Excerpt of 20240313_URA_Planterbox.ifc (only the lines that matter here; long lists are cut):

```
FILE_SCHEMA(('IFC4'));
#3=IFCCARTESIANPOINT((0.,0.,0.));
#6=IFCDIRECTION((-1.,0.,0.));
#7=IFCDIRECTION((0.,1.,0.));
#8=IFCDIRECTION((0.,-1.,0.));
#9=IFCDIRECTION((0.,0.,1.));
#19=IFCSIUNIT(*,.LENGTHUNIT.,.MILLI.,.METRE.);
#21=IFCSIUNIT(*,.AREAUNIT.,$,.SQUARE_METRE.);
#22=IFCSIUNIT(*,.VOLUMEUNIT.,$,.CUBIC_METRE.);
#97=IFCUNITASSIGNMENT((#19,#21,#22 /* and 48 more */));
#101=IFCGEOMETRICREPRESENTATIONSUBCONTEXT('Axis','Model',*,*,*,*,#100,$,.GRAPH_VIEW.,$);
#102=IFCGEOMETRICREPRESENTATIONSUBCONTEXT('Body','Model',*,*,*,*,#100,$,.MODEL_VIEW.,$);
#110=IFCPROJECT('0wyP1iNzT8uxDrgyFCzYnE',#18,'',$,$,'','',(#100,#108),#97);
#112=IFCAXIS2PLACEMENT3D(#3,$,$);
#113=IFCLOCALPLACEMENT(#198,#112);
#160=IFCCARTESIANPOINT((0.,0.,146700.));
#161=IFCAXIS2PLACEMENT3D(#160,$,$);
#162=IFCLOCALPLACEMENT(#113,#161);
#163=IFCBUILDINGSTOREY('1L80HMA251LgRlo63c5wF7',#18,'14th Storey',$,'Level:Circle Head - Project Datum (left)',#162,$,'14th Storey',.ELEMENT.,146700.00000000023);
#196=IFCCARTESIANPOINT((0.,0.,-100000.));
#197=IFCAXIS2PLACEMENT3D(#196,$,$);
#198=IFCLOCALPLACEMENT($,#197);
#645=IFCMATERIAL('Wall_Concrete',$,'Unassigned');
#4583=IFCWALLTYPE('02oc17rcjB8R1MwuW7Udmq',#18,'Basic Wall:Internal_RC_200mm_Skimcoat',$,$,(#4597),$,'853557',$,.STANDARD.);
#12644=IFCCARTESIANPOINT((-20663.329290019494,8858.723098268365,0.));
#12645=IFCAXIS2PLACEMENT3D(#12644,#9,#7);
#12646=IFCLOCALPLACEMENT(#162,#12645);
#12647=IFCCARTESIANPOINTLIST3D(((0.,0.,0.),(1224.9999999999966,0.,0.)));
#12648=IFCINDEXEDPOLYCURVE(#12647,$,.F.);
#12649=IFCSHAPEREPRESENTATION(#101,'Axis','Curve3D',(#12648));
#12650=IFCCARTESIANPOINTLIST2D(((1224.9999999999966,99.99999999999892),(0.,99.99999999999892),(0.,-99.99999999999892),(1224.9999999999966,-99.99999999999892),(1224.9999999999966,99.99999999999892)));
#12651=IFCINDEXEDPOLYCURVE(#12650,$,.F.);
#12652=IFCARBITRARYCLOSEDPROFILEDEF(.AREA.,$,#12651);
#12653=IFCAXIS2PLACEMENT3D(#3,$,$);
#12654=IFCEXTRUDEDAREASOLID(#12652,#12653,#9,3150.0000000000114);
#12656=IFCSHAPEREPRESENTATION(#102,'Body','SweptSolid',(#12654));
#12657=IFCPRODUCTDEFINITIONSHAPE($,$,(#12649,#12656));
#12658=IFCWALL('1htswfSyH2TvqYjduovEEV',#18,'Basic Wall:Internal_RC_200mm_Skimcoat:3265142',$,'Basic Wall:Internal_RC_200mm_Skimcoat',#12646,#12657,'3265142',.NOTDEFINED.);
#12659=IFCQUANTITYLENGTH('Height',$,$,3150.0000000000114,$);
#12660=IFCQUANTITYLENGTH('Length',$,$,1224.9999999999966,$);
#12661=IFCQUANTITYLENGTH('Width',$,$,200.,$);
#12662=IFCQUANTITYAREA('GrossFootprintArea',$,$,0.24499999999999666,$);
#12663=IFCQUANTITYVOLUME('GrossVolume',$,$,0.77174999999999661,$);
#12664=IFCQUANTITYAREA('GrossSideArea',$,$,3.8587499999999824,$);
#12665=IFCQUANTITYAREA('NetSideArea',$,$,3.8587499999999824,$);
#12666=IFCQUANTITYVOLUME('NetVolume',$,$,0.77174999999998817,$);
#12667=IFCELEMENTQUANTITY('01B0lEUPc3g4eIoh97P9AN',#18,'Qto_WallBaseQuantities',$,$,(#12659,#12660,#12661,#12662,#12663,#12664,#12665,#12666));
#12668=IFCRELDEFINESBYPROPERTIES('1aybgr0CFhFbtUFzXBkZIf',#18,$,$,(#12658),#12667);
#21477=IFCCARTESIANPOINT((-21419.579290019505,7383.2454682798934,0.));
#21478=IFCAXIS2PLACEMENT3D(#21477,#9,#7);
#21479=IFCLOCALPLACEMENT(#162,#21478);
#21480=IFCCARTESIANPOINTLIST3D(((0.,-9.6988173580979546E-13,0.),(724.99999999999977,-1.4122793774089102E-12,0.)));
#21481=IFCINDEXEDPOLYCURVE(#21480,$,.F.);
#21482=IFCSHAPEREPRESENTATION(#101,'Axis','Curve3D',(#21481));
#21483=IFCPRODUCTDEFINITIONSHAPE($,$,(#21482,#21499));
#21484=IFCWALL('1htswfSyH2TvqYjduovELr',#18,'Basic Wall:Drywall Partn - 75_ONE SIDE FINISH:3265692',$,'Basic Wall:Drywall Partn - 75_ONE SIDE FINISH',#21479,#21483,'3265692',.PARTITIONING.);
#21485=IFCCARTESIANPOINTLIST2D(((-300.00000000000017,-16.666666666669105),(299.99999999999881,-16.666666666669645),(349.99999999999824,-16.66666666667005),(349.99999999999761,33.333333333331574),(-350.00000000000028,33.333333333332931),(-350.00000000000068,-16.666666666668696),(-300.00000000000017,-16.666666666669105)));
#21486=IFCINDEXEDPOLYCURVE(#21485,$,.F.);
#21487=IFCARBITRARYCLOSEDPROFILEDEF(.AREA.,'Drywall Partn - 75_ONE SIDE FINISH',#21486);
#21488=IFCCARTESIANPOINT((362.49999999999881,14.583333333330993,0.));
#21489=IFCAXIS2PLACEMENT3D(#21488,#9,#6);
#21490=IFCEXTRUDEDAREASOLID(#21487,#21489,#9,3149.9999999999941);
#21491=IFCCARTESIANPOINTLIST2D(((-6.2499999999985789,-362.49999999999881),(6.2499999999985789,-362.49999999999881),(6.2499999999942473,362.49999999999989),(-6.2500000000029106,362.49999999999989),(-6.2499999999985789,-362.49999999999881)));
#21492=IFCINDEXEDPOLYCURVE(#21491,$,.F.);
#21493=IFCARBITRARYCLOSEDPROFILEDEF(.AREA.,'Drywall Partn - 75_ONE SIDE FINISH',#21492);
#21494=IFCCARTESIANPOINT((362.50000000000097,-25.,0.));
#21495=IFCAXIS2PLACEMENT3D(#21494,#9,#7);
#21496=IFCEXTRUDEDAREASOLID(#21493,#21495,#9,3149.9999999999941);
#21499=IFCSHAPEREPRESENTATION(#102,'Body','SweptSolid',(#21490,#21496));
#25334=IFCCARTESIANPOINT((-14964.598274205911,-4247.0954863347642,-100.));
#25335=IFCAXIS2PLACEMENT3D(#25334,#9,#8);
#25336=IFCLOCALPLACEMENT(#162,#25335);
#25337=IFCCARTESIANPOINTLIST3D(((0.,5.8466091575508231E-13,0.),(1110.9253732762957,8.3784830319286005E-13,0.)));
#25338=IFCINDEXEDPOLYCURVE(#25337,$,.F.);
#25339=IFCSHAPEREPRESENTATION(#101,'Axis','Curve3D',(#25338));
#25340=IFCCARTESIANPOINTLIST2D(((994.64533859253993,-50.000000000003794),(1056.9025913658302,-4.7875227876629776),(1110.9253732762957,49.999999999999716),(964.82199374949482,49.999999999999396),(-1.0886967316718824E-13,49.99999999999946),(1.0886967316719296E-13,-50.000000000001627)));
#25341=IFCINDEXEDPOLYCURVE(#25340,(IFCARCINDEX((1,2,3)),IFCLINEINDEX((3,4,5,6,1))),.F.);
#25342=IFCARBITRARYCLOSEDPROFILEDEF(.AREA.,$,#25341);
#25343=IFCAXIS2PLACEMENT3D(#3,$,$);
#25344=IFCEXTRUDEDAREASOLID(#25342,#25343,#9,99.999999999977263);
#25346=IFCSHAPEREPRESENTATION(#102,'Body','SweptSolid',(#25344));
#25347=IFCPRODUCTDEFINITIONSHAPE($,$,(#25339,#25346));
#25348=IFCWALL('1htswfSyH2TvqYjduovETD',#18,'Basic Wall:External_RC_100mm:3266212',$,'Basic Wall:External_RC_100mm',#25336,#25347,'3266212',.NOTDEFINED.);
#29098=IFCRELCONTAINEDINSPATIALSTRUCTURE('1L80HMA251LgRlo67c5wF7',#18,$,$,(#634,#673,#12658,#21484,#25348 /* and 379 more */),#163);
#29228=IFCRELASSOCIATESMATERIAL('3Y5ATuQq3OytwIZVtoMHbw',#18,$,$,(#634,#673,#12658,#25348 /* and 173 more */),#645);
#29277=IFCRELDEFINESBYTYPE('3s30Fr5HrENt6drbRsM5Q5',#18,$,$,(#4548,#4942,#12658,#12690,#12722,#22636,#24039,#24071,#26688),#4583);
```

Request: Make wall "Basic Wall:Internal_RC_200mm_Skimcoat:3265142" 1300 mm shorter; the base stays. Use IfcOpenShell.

```python
import ifcopenshell
import ifcopenshell.api.pset
import ifcopenshell.geom
import ifcopenshell.util.element
import ifcopenshell.util.representation
import ifcopenshell.util.shape
import ifcopenshell.util.unit

model = ifcopenshell.open("20240313_URA_Planterbox.ifc")
unit_scale = ifcopenshell.util.unit.calculate_unit_scale(model)
area_scale = ifcopenshell.util.unit.calculate_unit_scale(model, "AREAUNIT")
volume_scale = ifcopenshell.util.unit.calculate_unit_scale(model, "VOLUMEUNIT")
settings = ifcopenshell.geom.settings()


def volume(element):
    """Net volume in cubic metres, openings subtracted."""
    shape = ifcopenshell.geom.create_shape(settings, element)
    return ifcopenshell.util.shape.get_volume(shape.geometry)


wall = model.by_guid("1htswfSyH2TvqYjduovEEV")
before = volume(wall)

body = ifcopenshell.util.representation.get_representation(wall, "Model", "Body")
solid = body.Items[0]
old_height = solid.Depth
solid.Depth -= 1300.0
after = volume(wall)
thickness = 0.2  # wall thickness in metres

# Update the stored height, areas and volumes.
qto = model.by_id(ifcopenshell.util.element.get_pset(wall, "Qto_WallBaseQuantities", should_inherit=False)["id"])
ifcopenshell.api.pset.edit_qto(model, qto=qto, properties={
    "Height": solid.Depth,
    "GrossVolume": ifcopenshell.util.element.get_pset(wall, "Qto_WallBaseQuantities", "GrossVolume") * solid.Depth / old_height,
    "GrossSideArea": ifcopenshell.util.element.get_pset(wall, "Qto_WallBaseQuantities", "GrossSideArea") * solid.Depth / old_height,
    "NetSideArea": after / thickness / area_scale,
    "NetVolume": after / volume_scale,
})

print(f"height {old_height:g} -> {solid.Depth:g}, volume {before:.3f} -> {after:.3f} m3")

model.write("20240313_URA_Planterbox-out.ifc")
```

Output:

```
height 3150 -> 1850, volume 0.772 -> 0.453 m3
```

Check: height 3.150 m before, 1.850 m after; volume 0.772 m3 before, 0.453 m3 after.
